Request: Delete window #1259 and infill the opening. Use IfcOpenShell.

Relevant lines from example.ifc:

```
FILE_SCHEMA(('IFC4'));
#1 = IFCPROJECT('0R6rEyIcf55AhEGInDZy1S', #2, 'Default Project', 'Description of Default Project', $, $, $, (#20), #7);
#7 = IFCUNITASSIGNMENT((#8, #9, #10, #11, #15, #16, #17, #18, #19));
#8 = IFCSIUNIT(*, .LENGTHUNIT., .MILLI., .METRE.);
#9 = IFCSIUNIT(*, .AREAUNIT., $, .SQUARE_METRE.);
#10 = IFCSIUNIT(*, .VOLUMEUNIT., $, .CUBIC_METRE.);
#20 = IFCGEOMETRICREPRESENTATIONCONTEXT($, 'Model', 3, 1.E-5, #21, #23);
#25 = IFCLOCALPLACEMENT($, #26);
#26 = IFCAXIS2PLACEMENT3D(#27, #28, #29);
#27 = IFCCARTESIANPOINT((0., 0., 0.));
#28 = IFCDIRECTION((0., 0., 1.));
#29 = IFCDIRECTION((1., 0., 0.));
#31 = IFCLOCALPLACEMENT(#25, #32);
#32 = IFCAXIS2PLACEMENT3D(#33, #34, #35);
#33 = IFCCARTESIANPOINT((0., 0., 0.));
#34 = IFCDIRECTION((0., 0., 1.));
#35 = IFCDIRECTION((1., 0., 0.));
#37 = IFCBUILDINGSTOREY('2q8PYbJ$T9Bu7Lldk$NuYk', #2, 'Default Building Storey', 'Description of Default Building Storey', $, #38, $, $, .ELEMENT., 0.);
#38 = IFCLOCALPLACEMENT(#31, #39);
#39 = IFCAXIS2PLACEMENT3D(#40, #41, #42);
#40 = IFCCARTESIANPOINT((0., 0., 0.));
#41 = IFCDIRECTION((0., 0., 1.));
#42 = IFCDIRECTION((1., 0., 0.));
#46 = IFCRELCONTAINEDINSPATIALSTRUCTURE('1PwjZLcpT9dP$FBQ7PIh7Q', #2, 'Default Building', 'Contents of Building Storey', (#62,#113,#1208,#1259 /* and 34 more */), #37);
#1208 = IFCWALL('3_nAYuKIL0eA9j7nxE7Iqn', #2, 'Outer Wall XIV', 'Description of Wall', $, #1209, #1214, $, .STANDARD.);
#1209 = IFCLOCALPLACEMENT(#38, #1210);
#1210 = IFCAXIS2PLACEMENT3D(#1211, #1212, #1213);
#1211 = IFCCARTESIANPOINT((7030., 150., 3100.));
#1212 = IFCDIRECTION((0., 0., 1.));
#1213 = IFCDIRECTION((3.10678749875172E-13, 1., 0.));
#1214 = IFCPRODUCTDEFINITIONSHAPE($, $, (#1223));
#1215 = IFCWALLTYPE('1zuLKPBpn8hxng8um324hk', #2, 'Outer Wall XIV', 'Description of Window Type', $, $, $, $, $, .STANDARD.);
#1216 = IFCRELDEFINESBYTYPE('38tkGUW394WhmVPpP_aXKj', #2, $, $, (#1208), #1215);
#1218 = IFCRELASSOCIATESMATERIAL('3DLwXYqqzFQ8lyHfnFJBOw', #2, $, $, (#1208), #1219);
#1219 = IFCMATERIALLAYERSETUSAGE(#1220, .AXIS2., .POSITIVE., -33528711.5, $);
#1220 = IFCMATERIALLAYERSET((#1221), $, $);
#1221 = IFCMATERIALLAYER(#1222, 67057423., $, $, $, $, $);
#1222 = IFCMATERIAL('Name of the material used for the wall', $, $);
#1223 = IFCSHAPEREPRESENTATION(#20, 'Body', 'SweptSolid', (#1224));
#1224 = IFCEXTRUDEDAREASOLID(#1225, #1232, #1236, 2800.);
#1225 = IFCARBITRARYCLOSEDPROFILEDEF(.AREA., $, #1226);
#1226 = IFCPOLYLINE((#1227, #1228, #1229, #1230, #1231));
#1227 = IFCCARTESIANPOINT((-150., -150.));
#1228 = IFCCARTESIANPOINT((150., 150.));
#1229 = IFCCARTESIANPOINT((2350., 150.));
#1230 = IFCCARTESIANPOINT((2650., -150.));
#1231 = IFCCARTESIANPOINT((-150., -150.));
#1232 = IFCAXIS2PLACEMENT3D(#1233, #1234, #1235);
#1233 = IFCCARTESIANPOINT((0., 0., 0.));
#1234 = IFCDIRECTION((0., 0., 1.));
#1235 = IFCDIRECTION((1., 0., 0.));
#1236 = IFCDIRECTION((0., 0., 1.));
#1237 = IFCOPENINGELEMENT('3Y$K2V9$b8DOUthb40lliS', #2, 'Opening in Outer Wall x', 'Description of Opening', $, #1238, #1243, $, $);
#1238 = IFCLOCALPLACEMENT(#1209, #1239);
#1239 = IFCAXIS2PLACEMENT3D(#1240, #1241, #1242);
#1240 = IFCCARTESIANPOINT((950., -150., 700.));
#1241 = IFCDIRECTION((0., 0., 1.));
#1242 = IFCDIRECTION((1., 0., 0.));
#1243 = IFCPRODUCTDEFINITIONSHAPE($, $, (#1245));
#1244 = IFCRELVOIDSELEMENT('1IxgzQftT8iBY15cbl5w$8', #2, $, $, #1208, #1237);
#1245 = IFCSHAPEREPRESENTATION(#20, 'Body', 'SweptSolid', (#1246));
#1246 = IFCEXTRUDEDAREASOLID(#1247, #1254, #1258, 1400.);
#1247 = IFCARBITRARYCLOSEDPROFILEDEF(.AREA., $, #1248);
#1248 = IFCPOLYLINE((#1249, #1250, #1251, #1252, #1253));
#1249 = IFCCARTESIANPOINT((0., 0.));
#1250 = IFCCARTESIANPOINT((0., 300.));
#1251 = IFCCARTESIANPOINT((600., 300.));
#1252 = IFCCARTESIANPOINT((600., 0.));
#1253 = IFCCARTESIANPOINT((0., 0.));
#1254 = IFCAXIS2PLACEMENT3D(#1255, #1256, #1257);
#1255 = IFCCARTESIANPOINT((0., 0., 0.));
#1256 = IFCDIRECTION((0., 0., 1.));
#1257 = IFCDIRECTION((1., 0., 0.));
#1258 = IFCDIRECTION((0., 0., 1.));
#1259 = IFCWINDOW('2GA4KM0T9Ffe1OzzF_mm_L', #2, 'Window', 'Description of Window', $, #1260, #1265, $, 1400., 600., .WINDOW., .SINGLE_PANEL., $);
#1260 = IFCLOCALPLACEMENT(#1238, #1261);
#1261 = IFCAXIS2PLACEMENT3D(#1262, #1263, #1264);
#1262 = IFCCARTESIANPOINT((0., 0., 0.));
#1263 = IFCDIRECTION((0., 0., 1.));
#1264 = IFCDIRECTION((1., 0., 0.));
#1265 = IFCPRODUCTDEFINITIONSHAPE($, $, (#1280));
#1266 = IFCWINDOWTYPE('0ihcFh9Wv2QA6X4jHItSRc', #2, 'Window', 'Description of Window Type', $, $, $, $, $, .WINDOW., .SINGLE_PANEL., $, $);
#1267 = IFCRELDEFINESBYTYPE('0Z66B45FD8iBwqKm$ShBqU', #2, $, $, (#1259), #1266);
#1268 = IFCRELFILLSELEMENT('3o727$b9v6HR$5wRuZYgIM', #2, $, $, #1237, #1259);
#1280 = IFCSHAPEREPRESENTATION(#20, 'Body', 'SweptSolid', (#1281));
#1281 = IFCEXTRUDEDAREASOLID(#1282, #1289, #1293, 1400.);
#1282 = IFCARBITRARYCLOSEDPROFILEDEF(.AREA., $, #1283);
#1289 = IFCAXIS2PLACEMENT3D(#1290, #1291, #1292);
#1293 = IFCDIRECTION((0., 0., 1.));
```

```python
import ifcopenshell
import ifcopenshell.api.feature
import ifcopenshell.api.root
import ifcopenshell.geom
import ifcopenshell.util.shape

model = ifcopenshell.open("example.ifc")
settings = ifcopenshell.geom.settings()


def volume(element):
    """Net volume in cubic metres, openings subtracted."""
    shape = ifcopenshell.geom.create_shape(settings, element)
    return ifcopenshell.util.shape.get_volume(shape.geometry)


window = model.by_guid("2GA4KM0T9Ffe1OzzF_mm_L")
opening = window.FillsVoids[0].RelatingOpeningElement
wall = opening.VoidsElements[0].RelatingBuildingElement
before = volume(wall)

ifcopenshell.api.root.remove_product(model, product=window)
ifcopenshell.api.feature.remove_feature(model, feature=opening)

after = volume(wall)

print(f"wall volume {before:.3f} -> {after:.3f} m3")

model.write("example_edited.ifc")
```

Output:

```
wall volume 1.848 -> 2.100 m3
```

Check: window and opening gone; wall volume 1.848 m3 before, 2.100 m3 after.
